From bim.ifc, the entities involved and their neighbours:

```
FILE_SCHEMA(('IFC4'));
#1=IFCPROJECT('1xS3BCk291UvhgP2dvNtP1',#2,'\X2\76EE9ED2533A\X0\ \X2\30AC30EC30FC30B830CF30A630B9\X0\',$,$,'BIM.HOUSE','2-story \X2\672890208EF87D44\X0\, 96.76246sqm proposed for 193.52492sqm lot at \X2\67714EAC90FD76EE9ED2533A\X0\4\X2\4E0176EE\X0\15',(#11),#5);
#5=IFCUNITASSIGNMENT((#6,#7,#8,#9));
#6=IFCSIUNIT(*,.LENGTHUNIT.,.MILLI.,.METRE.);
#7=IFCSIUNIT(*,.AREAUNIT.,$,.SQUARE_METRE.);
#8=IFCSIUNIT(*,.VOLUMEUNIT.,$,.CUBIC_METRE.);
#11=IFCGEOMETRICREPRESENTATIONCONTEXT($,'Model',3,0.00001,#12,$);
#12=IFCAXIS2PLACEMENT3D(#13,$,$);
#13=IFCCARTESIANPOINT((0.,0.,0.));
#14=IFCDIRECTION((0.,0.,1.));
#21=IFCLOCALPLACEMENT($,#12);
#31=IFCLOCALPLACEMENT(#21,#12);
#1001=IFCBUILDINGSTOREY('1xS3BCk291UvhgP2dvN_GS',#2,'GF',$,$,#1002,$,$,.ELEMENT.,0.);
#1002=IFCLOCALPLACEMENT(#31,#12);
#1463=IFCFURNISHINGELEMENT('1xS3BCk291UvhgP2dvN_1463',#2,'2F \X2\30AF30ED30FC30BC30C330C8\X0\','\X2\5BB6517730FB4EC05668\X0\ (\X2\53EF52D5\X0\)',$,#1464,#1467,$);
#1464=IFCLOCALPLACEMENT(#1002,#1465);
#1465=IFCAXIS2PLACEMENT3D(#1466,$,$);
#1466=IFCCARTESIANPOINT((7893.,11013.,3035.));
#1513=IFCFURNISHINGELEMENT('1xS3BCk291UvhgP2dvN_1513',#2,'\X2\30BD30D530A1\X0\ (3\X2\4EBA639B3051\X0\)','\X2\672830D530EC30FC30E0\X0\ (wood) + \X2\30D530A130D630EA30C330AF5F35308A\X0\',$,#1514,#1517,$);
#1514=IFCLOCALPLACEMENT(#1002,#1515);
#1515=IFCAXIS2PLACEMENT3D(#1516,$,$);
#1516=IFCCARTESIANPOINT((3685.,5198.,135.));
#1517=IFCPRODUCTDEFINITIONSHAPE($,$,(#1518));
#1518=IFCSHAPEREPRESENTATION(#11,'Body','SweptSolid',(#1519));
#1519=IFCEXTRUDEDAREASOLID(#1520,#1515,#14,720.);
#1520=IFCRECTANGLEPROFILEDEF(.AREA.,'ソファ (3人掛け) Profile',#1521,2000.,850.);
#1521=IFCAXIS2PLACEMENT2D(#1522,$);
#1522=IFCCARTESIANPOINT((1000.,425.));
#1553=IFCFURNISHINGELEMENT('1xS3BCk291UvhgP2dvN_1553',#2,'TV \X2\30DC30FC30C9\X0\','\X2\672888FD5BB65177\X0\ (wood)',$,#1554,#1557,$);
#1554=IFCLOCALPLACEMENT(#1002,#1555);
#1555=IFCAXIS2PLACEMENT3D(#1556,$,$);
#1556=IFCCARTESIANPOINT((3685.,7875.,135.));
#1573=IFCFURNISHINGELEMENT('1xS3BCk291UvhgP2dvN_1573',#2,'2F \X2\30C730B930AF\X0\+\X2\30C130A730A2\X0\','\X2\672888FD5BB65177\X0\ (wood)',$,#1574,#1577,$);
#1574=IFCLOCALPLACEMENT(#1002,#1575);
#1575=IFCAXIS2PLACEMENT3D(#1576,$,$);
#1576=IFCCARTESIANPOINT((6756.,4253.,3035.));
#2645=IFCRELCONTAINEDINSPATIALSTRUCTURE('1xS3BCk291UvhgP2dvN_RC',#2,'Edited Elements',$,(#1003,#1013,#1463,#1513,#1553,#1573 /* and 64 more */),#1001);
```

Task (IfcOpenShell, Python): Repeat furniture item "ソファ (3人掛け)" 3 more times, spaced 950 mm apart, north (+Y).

```python
import numpy as np
import ifcopenshell
import ifcopenshell.api.geometry
import ifcopenshell.api.root
import ifcopenshell.util.element
import ifcopenshell.util.placement
import ifcopenshell.util.unit

model = ifcopenshell.open("bim.ifc")
unit_scale = ifcopenshell.util.unit.calculate_unit_scale(model)


def reuse_history(source, copy):
    """copy_class also copies each property set's owner history, people and application; keep the originals."""
    for rel in copy.IsDefinedBy:
        if rel.is_a("IfcRelDefinesByProperties") and (history := rel.RelatingPropertyDefinition.OwnerHistory):
            rel.RelatingPropertyDefinition.OwnerHistory = source.OwnerHistory
            ifcopenshell.util.element.remove_deep2(model, history)


source = model.by_guid("1xS3BCk291UvhgP2dvN_1513")
base = ifcopenshell.util.placement.get_local_placement(source.ObjectPlacement)
step = np.array([0.0, 1.0, 0.0]) * 0.95 / unit_scale

for i in range(1, 4):
    copy = ifcopenshell.api.root.copy_class(model, product=source)
    copy.Representation = ifcopenshell.util.element.copy_deep(
        model, source.Representation, exclude=["IfcGeometricRepresentationContext", "IfcRepresentationMap"]
    )
    reuse_history(source, copy)
    matrix = base.copy()
    matrix[:3, 3] += i * step
    print("added at", matrix[:3, 3].round(3) + 0.0)
    ifcopenshell.api.geometry.edit_object_placement(model, product=copy, matrix=matrix, is_si=False)

model.write("bim_v2.ifc")
```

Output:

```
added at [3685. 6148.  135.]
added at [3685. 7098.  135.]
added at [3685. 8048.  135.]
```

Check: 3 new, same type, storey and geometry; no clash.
